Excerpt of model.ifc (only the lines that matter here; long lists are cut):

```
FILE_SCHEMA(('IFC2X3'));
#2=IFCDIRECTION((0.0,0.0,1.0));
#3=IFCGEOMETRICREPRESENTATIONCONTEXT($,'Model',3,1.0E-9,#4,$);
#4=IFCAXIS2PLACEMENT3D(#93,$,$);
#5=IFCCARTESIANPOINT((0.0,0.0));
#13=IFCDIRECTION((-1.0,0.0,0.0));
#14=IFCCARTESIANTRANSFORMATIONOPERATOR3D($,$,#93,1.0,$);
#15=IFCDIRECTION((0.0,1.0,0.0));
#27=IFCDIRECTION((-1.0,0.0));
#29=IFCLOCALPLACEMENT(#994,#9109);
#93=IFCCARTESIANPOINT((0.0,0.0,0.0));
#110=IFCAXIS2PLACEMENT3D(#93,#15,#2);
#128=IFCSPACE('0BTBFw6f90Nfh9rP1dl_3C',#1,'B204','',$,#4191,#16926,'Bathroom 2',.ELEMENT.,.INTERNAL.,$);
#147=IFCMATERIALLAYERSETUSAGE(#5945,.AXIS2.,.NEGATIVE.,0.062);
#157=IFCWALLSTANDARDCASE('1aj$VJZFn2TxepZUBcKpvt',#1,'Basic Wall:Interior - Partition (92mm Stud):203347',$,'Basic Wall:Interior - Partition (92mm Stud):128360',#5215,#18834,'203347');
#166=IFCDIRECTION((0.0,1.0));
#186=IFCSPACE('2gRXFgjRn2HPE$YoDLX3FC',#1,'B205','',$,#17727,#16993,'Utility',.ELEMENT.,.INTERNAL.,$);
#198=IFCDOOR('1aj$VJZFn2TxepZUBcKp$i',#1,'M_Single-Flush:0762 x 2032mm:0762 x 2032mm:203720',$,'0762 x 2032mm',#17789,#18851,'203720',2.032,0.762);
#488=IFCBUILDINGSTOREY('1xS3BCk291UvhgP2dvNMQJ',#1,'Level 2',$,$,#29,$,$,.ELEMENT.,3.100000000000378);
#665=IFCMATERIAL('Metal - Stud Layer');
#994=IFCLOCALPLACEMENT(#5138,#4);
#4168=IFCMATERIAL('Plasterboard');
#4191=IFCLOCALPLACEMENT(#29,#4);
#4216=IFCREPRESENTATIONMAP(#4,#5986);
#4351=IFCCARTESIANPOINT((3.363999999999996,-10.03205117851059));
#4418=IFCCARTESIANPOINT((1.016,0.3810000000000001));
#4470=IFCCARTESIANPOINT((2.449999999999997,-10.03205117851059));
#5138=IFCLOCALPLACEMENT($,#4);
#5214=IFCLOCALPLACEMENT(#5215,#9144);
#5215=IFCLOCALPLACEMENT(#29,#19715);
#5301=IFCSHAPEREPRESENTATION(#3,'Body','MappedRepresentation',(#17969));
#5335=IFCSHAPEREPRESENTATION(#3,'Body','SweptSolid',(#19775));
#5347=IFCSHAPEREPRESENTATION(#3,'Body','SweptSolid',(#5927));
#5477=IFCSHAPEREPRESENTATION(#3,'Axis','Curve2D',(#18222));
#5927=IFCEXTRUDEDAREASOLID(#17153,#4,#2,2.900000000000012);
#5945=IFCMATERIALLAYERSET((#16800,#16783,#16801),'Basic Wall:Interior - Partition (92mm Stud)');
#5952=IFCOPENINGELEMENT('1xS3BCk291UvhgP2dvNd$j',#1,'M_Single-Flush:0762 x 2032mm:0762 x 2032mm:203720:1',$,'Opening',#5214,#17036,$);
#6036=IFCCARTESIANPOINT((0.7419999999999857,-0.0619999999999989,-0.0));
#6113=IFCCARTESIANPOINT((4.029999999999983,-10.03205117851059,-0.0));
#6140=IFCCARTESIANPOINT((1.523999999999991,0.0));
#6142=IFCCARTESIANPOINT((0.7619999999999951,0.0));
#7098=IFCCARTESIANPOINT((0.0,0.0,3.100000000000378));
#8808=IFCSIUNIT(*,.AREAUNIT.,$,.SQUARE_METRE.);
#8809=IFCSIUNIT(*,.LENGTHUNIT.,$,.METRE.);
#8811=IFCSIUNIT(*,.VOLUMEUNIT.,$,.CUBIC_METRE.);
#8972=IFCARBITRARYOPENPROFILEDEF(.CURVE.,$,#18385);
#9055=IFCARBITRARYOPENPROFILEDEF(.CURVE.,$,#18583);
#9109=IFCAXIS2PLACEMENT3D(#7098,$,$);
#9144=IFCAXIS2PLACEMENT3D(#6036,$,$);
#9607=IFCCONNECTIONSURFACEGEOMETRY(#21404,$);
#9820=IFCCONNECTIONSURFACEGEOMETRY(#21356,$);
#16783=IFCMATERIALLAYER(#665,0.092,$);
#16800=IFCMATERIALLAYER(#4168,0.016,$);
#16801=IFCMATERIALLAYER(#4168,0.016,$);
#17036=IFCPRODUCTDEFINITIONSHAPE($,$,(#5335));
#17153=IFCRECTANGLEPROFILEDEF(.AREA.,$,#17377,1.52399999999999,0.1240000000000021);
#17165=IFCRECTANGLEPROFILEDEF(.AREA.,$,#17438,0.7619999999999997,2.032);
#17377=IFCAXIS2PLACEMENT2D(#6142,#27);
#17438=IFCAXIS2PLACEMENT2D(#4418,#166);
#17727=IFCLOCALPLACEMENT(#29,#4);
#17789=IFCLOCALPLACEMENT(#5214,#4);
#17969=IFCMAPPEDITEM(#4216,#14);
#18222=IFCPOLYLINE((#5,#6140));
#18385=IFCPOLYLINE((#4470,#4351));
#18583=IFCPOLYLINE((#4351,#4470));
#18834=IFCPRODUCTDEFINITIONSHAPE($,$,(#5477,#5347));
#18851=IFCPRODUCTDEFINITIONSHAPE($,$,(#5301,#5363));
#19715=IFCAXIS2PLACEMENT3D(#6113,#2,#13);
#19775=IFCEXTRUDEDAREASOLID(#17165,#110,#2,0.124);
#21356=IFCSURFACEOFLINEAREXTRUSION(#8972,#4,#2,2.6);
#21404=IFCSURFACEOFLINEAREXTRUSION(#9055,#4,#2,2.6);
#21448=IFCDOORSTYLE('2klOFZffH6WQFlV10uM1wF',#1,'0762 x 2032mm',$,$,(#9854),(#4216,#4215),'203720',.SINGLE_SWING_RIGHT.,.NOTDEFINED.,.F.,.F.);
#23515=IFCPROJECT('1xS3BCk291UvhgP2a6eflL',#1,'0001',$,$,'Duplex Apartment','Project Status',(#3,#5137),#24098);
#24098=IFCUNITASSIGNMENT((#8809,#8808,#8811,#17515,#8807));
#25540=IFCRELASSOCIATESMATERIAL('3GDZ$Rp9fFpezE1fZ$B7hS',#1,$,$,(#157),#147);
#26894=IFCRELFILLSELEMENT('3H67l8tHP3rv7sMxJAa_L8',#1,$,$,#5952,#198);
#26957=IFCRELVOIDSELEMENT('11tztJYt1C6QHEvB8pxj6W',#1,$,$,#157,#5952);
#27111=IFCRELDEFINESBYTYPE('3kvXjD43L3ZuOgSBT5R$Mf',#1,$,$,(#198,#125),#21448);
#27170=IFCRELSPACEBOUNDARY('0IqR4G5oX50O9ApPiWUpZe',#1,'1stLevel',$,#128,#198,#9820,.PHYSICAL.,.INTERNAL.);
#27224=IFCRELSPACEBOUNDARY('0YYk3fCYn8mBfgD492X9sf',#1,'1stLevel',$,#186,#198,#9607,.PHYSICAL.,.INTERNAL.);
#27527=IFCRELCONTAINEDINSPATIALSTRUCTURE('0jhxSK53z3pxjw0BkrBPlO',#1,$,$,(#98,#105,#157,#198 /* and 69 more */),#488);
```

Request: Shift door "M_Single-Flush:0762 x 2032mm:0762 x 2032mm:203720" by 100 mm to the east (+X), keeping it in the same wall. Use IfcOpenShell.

```python
import numpy as np
import ifcopenshell
import ifcopenshell.api.geometry
import ifcopenshell.util.placement
import ifcopenshell.util.unit

model = ifcopenshell.open("model.ifc")
unit_scale = ifcopenshell.util.unit.calculate_unit_scale(model)

door = model.by_guid("1aj$VJZFn2TxepZUBcKp$i")
opening = door.FillsVoids[0].RelatingOpeningElement
wall = opening.VoidsElements[0].RelatingBuildingElement

wall_matrix = ifcopenshell.util.placement.get_local_placement(wall.ObjectPlacement)
shift = wall_matrix[:3, 0] * -0.1 / unit_scale
before = ifcopenshell.util.placement.get_local_placement(door.ObjectPlacement)[:3, 3].copy()

# The door is placed relative to its opening, so it follows when the opening moves.
matrix = ifcopenshell.util.placement.get_local_placement(opening.ObjectPlacement)
matrix[:3, 3] += shift
ifcopenshell.api.geometry.edit_object_placement(
    model, product=opening, matrix=matrix, is_si=False, should_transform_children=True
)

# Space boundary surfaces are stored in each space's coordinates; move them too.
for rel in door.ProvidesBoundaries:
    if not rel.ConnectionGeometry:
        continue
    surface = rel.ConnectionGeometry.SurfaceOnRelatingElement
    space_matrix = ifcopenshell.util.placement.get_local_placement(rel.RelatingSpace.ObjectPlacement)
    point = np.array(surface.Position.Location.Coordinates) + space_matrix[:3, :3].T @ shift
    surface.Position = model.createIfcAxis2Placement3D(
        model.createIfcCartesianPoint(point.tolist()), surface.Position.Axis, surface.Position.RefDirection
    )

after = ifcopenshell.util.placement.get_local_placement(door.ObjectPlacement)[:3, 3]
print("door moved by", (after - before).round(3) + 0.0)

model.write("model_edited.ifc")
```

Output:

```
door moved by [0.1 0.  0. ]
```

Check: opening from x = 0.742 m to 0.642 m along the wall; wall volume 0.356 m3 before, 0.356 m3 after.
